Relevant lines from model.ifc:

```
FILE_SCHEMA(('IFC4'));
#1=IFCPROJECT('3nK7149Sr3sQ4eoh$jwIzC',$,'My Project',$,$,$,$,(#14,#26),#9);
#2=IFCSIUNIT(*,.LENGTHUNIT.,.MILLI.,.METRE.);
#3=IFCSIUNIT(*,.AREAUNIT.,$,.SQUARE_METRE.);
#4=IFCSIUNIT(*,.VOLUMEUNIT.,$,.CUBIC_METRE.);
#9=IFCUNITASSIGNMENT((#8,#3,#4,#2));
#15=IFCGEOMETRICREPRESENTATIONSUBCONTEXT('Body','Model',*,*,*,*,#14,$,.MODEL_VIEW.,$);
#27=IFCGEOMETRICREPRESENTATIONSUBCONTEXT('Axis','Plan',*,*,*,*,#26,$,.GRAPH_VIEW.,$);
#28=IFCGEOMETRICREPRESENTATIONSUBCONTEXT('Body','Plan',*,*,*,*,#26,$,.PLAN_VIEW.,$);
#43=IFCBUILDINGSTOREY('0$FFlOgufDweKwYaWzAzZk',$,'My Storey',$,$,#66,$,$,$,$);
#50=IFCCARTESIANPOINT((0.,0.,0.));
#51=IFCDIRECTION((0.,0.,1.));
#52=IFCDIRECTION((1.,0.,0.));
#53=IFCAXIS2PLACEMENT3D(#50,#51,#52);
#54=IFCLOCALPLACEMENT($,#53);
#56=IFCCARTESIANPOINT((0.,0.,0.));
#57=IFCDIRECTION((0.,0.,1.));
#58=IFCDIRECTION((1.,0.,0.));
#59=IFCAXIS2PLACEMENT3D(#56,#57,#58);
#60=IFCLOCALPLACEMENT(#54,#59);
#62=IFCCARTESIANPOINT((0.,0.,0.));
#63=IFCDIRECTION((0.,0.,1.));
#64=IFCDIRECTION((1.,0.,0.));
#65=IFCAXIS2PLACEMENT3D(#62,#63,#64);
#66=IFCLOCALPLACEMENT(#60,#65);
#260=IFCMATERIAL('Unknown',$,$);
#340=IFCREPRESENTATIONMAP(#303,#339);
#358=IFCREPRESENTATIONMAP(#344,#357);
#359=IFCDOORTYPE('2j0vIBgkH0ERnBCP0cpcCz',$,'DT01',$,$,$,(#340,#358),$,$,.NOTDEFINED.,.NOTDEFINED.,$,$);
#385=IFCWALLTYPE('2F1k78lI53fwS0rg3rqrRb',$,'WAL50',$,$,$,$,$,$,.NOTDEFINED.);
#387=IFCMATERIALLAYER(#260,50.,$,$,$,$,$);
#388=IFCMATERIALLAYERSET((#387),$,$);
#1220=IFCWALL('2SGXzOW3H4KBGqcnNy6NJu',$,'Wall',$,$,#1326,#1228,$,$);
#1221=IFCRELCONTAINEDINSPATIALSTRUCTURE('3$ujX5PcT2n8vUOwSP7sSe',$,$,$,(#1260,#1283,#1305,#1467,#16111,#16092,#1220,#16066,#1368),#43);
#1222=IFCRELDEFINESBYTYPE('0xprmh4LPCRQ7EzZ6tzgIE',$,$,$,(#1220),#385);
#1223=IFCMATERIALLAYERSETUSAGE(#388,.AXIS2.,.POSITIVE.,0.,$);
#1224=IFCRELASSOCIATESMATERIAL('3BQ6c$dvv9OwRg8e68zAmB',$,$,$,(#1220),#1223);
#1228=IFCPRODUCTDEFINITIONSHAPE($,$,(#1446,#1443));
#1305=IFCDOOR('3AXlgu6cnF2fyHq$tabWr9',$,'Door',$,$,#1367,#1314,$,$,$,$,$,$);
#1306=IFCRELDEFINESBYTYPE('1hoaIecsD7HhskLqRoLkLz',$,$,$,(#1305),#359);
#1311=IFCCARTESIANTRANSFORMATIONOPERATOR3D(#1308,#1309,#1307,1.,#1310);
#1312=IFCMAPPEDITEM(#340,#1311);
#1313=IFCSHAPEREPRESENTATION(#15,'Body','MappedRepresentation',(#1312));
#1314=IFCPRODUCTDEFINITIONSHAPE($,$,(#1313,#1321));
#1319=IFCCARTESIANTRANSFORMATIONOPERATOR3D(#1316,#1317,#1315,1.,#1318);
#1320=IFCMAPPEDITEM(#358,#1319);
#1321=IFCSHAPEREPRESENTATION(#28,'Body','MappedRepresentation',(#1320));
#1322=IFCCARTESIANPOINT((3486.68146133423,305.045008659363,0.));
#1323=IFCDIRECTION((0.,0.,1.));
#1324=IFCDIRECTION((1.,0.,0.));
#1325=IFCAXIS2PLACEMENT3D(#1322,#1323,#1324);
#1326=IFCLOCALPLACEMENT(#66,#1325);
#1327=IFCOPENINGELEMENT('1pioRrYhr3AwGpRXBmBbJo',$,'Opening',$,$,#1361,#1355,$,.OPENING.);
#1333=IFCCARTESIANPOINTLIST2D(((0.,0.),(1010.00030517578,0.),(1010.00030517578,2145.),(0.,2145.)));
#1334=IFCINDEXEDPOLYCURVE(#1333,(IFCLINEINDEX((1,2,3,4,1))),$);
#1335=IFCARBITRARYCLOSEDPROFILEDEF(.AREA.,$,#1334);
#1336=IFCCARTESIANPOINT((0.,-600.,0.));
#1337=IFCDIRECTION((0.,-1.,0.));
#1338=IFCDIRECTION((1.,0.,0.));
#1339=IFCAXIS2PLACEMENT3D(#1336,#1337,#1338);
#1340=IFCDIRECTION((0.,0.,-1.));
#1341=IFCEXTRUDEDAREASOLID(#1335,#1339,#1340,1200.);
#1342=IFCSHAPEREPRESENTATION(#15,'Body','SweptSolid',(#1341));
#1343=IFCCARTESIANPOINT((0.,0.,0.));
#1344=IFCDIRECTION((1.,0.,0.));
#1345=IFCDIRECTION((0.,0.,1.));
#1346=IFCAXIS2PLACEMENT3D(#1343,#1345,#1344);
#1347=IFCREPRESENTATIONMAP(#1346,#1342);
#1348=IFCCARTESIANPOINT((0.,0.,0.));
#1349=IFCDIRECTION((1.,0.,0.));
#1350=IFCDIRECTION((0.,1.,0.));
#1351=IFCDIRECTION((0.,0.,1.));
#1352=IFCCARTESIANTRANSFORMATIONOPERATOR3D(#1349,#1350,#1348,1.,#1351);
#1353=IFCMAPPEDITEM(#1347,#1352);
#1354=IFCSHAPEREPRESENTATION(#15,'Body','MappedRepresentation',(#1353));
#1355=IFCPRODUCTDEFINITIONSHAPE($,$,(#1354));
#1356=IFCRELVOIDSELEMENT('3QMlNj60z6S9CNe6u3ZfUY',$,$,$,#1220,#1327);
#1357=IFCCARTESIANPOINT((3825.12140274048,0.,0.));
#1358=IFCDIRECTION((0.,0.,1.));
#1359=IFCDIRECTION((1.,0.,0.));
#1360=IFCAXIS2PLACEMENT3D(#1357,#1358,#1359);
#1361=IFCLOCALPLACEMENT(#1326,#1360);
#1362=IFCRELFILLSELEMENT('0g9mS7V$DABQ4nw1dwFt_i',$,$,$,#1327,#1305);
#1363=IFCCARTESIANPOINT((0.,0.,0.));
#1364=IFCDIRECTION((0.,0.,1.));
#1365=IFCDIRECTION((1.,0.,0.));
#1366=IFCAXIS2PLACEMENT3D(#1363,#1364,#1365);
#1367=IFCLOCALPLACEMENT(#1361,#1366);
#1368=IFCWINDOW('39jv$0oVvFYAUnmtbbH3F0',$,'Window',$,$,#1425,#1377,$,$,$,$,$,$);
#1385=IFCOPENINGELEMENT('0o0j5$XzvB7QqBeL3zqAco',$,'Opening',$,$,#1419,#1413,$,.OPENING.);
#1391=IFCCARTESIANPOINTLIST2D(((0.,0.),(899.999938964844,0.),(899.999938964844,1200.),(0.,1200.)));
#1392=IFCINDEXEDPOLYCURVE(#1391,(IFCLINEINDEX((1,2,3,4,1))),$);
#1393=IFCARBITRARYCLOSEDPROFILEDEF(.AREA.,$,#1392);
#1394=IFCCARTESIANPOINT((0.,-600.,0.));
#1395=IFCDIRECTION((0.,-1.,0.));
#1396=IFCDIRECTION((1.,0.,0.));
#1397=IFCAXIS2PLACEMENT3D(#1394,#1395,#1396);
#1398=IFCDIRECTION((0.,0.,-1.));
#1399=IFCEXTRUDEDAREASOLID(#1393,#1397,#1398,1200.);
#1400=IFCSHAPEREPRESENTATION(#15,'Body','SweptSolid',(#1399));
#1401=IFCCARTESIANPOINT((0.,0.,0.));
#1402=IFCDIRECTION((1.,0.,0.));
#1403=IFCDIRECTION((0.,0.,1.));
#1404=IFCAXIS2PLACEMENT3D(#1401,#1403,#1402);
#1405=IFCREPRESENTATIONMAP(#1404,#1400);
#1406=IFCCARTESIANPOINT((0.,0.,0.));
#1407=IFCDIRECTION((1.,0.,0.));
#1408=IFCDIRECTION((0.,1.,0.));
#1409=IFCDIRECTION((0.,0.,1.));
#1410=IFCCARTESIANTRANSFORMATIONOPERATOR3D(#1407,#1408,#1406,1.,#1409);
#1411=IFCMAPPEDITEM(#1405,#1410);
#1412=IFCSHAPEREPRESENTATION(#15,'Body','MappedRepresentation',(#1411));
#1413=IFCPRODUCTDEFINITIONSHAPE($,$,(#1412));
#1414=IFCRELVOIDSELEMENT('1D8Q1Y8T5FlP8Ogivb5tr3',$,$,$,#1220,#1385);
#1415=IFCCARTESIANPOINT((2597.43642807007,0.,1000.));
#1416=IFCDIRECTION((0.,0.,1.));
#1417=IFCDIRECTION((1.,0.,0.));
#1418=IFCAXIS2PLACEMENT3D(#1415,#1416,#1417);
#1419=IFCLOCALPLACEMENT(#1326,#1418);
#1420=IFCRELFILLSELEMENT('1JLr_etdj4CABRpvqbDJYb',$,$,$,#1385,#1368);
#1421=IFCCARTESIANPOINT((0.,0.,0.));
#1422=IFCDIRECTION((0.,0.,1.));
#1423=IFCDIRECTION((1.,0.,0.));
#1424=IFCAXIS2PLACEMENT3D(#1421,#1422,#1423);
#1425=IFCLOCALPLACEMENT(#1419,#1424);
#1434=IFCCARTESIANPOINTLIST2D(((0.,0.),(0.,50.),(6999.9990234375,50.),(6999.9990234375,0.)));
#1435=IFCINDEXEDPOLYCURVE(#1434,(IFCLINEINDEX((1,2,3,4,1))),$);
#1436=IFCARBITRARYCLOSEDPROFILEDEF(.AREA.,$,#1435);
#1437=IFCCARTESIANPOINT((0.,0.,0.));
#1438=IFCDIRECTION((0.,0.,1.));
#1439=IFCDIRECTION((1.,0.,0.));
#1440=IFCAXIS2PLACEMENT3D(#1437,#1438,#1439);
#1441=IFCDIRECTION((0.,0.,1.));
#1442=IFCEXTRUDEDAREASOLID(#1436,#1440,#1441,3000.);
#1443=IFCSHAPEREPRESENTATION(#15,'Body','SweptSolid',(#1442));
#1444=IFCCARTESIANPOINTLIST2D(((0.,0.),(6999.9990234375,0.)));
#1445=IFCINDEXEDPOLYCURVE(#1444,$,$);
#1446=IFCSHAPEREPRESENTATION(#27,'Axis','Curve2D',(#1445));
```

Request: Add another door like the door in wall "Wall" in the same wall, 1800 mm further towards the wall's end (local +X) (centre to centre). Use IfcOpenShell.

```python
import ifcopenshell
import ifcopenshell.api.feature
import ifcopenshell.api.geometry
import ifcopenshell.api.root
import ifcopenshell.geom
import ifcopenshell.util.element
import ifcopenshell.util.placement
import ifcopenshell.util.shape

model = ifcopenshell.open("model.ifc")
settings = ifcopenshell.geom.settings()


def volume(element):
    """Net volume in cubic metres, openings subtracted."""
    shape = ifcopenshell.geom.create_shape(settings, element)
    return ifcopenshell.util.shape.get_volume(shape.geometry)


door = model.by_guid("3AXlgu6cnF2fyHq$tabWr9")
opening = door.FillsVoids[0].RelatingOpeningElement
wall = opening.VoidsElements[0].RelatingBuildingElement
before = volume(wall)
shift = ifcopenshell.util.placement.get_local_placement(wall.ObjectPlacement)[:3, 0] * 1800.0

# copy_class copies the void relationship, type, container and properties, but no geometry.
new_opening = ifcopenshell.api.root.copy_class(model, product=opening)
new_opening.Representation = ifcopenshell.util.element.copy_deep(
    model, opening.Representation, exclude=["IfcGeometricRepresentationContext", "IfcRepresentationMap"]
)
new_door = ifcopenshell.api.root.copy_class(model, product=door)
new_door.Representation = ifcopenshell.util.element.copy_deep(
    model, door.Representation, exclude=["IfcGeometricRepresentationContext", "IfcRepresentationMap"]
)
ifcopenshell.api.feature.add_filling(model, opening=new_opening, element=new_door)

for old, new in ((opening, new_opening), (door, new_door)):
    matrix = ifcopenshell.util.placement.get_local_placement(old.ObjectPlacement)
    matrix[:3, 3] += shift
    ifcopenshell.api.geometry.edit_object_placement(model, product=new, matrix=matrix, is_si=False)

after = volume(wall)

print(f"wall volume {before:.3f} -> {after:.3f} m3")

model.write("model-out.ifc")
```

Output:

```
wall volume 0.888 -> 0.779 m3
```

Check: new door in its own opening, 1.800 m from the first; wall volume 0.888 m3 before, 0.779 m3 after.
